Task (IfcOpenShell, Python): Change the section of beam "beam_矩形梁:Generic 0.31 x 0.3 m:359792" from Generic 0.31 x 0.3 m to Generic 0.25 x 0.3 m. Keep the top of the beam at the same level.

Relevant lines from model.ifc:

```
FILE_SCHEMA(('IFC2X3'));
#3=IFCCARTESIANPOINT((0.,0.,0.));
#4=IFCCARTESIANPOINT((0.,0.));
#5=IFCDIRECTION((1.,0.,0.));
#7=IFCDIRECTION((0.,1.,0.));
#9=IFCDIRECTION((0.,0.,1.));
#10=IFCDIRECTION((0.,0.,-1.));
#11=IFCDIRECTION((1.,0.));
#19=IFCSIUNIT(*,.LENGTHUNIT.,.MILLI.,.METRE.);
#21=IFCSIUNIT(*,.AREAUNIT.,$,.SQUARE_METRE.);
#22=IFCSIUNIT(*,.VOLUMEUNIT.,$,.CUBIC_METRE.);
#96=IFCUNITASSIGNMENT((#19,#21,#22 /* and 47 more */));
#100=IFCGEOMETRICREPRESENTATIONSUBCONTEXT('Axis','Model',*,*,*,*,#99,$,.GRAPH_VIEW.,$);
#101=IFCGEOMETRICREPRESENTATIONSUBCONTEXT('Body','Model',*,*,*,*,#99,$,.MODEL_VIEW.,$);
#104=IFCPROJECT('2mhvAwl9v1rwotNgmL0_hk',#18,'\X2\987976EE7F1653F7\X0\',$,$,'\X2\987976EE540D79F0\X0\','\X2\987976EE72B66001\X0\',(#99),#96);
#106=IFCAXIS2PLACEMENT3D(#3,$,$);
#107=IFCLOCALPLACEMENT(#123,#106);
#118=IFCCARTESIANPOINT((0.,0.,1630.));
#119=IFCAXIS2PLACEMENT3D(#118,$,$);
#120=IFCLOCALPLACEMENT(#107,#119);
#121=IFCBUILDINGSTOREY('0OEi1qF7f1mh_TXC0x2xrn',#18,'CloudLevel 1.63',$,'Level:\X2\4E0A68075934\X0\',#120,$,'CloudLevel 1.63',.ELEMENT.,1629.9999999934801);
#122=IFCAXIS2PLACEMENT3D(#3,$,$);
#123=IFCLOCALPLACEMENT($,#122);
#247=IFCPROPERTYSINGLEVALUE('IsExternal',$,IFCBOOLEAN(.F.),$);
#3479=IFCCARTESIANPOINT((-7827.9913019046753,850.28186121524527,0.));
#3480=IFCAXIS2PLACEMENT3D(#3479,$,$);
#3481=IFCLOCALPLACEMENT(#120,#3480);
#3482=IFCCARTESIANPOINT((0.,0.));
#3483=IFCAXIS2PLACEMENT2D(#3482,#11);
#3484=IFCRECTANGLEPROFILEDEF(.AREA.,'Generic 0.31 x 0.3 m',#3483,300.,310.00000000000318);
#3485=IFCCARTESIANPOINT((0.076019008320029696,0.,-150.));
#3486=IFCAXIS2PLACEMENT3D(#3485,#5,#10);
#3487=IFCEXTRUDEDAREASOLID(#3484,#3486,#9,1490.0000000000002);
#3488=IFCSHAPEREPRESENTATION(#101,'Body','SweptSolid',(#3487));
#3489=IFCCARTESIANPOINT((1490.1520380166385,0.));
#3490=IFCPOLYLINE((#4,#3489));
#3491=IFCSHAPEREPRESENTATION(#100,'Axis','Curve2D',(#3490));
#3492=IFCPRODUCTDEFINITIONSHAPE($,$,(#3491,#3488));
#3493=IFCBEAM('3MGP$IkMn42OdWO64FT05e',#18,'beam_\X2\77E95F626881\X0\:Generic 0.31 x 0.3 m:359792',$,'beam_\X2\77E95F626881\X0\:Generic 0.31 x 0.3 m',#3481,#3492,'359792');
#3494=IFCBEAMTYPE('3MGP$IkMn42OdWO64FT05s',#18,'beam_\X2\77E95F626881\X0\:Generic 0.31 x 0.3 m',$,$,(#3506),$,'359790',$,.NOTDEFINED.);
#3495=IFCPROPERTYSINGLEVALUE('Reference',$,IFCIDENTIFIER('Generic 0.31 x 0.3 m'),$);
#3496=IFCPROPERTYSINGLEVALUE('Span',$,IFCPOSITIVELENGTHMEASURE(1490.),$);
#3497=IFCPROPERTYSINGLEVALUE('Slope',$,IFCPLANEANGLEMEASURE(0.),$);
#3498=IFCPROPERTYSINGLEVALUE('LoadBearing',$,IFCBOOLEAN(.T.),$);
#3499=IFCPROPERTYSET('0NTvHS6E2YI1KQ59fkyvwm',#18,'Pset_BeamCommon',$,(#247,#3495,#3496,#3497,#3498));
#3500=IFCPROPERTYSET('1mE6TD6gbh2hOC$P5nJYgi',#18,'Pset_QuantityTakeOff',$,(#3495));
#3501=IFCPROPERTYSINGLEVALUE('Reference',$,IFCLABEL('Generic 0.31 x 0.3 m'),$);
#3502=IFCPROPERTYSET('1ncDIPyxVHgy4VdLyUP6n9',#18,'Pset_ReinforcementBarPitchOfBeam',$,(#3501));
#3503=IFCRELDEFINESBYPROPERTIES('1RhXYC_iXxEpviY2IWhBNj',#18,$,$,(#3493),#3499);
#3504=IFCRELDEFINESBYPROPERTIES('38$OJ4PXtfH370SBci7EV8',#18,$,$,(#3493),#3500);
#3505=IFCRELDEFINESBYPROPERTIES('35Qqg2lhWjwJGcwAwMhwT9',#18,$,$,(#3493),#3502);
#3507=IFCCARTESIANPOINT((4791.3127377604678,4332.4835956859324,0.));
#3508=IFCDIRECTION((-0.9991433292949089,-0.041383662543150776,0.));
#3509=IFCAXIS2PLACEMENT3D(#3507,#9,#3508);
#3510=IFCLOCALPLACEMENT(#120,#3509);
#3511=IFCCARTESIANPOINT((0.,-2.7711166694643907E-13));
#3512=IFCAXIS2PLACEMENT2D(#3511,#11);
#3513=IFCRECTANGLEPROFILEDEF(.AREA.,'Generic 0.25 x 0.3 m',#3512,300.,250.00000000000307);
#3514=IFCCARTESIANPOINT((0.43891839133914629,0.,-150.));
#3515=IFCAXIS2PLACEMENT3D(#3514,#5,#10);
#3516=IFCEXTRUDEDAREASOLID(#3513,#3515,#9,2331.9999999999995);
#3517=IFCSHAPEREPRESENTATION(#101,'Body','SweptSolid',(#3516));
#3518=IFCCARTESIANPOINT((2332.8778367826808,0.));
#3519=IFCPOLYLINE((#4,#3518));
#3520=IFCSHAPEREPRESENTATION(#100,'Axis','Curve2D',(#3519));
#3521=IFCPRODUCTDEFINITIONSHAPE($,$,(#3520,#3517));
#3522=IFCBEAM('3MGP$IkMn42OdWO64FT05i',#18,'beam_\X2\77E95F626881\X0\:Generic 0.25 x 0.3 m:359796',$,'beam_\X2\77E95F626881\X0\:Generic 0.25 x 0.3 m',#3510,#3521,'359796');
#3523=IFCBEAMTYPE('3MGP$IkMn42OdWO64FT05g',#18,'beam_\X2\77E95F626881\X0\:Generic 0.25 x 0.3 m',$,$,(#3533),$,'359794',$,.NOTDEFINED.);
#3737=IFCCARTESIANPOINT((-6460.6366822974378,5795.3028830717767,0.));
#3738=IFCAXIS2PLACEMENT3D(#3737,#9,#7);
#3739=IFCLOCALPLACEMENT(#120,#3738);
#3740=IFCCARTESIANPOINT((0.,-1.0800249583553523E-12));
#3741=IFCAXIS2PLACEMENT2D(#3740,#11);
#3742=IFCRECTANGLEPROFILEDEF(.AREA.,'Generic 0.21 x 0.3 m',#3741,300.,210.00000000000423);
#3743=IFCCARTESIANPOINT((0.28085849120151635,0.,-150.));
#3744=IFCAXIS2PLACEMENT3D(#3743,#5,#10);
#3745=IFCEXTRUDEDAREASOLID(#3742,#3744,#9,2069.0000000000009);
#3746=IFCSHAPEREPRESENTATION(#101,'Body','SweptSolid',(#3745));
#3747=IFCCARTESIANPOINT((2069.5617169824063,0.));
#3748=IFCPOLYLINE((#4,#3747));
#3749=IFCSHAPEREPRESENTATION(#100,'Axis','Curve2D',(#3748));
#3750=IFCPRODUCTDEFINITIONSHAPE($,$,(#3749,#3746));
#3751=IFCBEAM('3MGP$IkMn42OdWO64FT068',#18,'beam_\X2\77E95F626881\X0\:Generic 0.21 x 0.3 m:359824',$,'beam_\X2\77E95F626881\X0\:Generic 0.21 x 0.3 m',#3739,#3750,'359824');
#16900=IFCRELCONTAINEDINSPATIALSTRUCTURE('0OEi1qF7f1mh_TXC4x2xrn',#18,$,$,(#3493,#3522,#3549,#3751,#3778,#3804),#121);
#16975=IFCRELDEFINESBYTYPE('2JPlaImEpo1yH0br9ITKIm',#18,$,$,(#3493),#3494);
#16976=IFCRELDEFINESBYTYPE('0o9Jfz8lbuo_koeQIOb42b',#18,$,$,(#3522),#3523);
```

```python
import ifcopenshell
import ifcopenshell.api.pset
import ifcopenshell.api.type
import ifcopenshell.util.element
import ifcopenshell.util.representation

model = ifcopenshell.open("model.ifc")

member = model.by_id(3493)
source = next(p for p in model.by_type("IfcRectangleProfileDef") if p.ProfileName == "Generic 0.25 x 0.3 m")

body = ifcopenshell.util.representation.get_representation(member, "Model", "Body")
solid = body.Items[0]
old_profile = solid.SweptArea

# Copy the section's sizes but keep this member's own profile position.
profile = ifcopenshell.util.element.copy(model, source)
# Profiles are centred, so shift by half the change in depth to hold the top.
shift = (old_profile.XDim - profile.XDim) / 2
x, y = old_profile.Position.Location.Coordinates
up = (-1.0, 0.0)  # upwards, in the solid's own plane
location = model.createIfcCartesianPoint((x + up[0] * shift, y + up[1] * shift))
profile.Position = model.createIfcAxis2Placement2D(location, old_profile.Position.RefDirection)
solid.SweptArea = profile
if not model.get_total_inverses(old_profile):
    ifcopenshell.util.element.remove_deep2(model, old_profile)

new_type = model.by_guid("3MGP$IkMn42OdWO64FT05g")
ifcopenshell.api.type.assign_type(
    model, related_objects=[member], relating_type=new_type, should_map_representations=False
)
member.Name = member.Name.replace("Generic 0.31 x 0.3 m", "Generic 0.25 x 0.3 m")
member.ObjectType = "beam_矩形梁:Generic 0.25 x 0.3 m"
pset = model.by_id(ifcopenshell.util.element.get_pset(member, "Pset_BeamCommon", should_inherit=False)["id"])
ifcopenshell.api.pset.edit_pset(model, pset=pset, properties={"Reference": "Generic 0.25 x 0.3 m"})
pset = model.by_id(ifcopenshell.util.element.get_pset(member, "Pset_QuantityTakeOff", should_inherit=False)["id"])
ifcopenshell.api.pset.edit_pset(model, pset=pset, properties={"Reference": "Generic 0.25 x 0.3 m"})
pset = model.by_id(ifcopenshell.util.element.get_pset(member, "Pset_ReinforcementBarPitchOfBeam", should_inherit=False)["id"])
ifcopenshell.api.pset.edit_pset(model, pset=pset, properties={"Reference": "Generic 0.25 x 0.3 m"})

print(solid.SweptArea)

model.write("model_rev.ifc")
```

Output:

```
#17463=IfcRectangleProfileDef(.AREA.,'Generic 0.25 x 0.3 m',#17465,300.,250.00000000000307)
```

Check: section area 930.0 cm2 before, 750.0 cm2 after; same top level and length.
